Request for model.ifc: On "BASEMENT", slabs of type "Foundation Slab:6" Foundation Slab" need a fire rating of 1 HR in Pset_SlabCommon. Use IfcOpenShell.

First a look at what the model holds.

```python
import ifcopenshell
import ifcopenshell.util.element

model = ifcopenshell.open("model.ifc")
print(model.schema)
storey = next(s for s in model.by_type("IfcBuildingStorey") if s.Name == "BASEMENT")
slabs = [e for e in ifcopenshell.util.element.get_decomposition(storey) if e.is_a("IfcSlab")]
seen = {}
for e in slabs:
    element_type = ifcopenshell.util.element.get_type(e)
    key = (element_type.Name if element_type != e and element_type else None, ifcopenshell.util.element.get_pset(e, "Pset_SlabCommon", "FireRating"))
    seen[key] = seen.get(key, 0) + 1
for (name, value), count in sorted(seen.items(), key=str):
    print(count, "x", name, "|", value)
```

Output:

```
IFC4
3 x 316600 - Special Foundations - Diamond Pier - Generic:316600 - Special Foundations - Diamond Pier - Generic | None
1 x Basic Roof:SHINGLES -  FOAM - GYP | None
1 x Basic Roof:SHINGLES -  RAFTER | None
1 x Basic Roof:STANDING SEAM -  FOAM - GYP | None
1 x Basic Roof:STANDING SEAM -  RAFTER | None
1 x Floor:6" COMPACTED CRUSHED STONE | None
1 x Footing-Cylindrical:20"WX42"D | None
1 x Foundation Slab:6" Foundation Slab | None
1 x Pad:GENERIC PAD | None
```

```python
import ifcopenshell
import ifcopenshell.api.pset
import ifcopenshell.util.element

model = ifcopenshell.open("model.ifc")

storey = next(s for s in model.by_type("IfcBuildingStorey") if s.Name == "BASEMENT")
slabs = [e for e in ifcopenshell.util.element.get_decomposition(storey) if e.is_a("IfcSlab")]

count = 0
for e in slabs:
    element_type = ifcopenshell.util.element.get_type(e)
    if element_type in (None, e) or element_type.Name != 'Foundation Slab:6" Foundation Slab':
        continue
    # add_pset returns the element's existing set when there is one.
    pset = ifcopenshell.api.pset.add_pset(model, product=e, name="Pset_SlabCommon")
    ifcopenshell.api.pset.edit_pset(model, pset=pset, properties={"FireRating": "1 HR"})
    count += 1

print(count, "slabs updated")

model.write("model_edited.ifc")
```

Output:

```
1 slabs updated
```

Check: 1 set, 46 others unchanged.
